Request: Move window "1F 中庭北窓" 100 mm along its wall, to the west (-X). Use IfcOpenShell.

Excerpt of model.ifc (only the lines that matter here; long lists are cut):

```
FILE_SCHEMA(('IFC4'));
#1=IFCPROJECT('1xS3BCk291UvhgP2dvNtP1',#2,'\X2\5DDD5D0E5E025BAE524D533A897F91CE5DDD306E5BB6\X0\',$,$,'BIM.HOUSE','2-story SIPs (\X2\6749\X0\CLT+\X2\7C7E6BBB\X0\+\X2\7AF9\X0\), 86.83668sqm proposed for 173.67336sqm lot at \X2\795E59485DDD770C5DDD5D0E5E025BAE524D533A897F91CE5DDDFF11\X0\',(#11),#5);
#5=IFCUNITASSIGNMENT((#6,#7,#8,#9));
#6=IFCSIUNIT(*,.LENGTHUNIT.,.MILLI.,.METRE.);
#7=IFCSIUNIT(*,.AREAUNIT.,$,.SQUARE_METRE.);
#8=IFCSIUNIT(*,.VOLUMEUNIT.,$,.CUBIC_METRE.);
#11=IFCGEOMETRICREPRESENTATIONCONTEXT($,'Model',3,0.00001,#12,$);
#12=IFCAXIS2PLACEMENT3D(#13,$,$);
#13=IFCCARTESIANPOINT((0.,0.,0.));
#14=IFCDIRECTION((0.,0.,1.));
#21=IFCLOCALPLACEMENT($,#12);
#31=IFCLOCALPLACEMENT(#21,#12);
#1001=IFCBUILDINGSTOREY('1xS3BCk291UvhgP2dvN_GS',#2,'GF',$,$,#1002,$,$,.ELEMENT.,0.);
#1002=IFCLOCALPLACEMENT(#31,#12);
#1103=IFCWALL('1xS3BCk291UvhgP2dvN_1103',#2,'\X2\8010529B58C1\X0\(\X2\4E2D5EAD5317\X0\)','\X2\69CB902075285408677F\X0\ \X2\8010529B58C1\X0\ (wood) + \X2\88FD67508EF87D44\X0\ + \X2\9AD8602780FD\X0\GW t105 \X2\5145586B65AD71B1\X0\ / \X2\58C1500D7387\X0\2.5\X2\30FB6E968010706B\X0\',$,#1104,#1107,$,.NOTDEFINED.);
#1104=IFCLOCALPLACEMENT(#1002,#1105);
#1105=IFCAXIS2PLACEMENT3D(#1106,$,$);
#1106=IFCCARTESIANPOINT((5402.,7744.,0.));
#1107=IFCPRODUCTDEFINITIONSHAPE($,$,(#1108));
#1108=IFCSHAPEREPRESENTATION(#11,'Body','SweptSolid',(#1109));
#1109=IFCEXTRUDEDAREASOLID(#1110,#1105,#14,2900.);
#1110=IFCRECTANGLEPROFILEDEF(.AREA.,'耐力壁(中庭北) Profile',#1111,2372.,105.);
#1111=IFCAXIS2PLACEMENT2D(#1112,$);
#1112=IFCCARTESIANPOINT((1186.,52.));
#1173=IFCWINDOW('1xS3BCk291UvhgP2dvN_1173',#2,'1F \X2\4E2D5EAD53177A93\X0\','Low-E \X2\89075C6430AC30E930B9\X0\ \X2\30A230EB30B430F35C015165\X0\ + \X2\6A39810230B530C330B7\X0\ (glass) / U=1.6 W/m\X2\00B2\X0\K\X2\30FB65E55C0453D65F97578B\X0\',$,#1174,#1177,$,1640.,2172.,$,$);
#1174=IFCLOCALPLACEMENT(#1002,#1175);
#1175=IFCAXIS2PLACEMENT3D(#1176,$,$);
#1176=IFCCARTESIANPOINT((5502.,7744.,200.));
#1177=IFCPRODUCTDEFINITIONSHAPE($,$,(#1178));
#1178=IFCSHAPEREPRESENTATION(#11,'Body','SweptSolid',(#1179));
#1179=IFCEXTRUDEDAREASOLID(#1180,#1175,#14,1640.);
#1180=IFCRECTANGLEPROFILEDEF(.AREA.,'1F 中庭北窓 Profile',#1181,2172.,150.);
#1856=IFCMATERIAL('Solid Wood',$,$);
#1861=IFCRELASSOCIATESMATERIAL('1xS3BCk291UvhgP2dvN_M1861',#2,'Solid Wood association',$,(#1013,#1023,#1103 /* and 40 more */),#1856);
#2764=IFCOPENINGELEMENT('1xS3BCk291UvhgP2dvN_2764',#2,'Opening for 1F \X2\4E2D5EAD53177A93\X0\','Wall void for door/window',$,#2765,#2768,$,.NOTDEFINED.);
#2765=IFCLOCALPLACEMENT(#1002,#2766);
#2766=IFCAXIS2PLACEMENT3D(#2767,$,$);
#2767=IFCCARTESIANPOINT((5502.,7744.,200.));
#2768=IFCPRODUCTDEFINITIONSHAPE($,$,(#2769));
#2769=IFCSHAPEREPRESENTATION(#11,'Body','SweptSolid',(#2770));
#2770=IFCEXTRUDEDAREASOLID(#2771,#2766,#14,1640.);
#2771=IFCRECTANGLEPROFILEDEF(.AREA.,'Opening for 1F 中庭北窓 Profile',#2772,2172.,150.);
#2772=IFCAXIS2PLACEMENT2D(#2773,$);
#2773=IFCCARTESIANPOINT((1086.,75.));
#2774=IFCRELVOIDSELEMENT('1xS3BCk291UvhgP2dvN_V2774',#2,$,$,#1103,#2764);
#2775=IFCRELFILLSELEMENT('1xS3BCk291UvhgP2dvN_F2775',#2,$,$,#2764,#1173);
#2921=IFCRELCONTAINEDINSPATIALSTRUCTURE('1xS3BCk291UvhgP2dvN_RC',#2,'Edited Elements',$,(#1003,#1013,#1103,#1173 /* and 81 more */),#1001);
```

```python
import ifcopenshell
import ifcopenshell.api.geometry
import ifcopenshell.util.placement
import ifcopenshell.util.unit

model = ifcopenshell.open("model.ifc")
unit_scale = ifcopenshell.util.unit.calculate_unit_scale(model)

window = model.by_guid("1xS3BCk291UvhgP2dvN_1173")
opening = window.FillsVoids[0].RelatingOpeningElement
wall = opening.VoidsElements[0].RelatingBuildingElement

wall_matrix = ifcopenshell.util.placement.get_local_placement(wall.ObjectPlacement)
shift = wall_matrix[:3, 0] * -0.1 / unit_scale
before = ifcopenshell.util.placement.get_local_placement(window.ObjectPlacement)[:3, 3].copy()

# The window is not placed relative to its opening, so move both.
for product in (opening, window):
    matrix = ifcopenshell.util.placement.get_local_placement(product.ObjectPlacement)
    matrix[:3, 3] += shift
    ifcopenshell.api.geometry.edit_object_placement(model, product=product, matrix=matrix, is_si=False)

after = ifcopenshell.util.placement.get_local_placement(window.ObjectPlacement)[:3, 3]
print("window moved by", (after - before).round(3) + 0.0)

model.write("model_edited.ifc")
```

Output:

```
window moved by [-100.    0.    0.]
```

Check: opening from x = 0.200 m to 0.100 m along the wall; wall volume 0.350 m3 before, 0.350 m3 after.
